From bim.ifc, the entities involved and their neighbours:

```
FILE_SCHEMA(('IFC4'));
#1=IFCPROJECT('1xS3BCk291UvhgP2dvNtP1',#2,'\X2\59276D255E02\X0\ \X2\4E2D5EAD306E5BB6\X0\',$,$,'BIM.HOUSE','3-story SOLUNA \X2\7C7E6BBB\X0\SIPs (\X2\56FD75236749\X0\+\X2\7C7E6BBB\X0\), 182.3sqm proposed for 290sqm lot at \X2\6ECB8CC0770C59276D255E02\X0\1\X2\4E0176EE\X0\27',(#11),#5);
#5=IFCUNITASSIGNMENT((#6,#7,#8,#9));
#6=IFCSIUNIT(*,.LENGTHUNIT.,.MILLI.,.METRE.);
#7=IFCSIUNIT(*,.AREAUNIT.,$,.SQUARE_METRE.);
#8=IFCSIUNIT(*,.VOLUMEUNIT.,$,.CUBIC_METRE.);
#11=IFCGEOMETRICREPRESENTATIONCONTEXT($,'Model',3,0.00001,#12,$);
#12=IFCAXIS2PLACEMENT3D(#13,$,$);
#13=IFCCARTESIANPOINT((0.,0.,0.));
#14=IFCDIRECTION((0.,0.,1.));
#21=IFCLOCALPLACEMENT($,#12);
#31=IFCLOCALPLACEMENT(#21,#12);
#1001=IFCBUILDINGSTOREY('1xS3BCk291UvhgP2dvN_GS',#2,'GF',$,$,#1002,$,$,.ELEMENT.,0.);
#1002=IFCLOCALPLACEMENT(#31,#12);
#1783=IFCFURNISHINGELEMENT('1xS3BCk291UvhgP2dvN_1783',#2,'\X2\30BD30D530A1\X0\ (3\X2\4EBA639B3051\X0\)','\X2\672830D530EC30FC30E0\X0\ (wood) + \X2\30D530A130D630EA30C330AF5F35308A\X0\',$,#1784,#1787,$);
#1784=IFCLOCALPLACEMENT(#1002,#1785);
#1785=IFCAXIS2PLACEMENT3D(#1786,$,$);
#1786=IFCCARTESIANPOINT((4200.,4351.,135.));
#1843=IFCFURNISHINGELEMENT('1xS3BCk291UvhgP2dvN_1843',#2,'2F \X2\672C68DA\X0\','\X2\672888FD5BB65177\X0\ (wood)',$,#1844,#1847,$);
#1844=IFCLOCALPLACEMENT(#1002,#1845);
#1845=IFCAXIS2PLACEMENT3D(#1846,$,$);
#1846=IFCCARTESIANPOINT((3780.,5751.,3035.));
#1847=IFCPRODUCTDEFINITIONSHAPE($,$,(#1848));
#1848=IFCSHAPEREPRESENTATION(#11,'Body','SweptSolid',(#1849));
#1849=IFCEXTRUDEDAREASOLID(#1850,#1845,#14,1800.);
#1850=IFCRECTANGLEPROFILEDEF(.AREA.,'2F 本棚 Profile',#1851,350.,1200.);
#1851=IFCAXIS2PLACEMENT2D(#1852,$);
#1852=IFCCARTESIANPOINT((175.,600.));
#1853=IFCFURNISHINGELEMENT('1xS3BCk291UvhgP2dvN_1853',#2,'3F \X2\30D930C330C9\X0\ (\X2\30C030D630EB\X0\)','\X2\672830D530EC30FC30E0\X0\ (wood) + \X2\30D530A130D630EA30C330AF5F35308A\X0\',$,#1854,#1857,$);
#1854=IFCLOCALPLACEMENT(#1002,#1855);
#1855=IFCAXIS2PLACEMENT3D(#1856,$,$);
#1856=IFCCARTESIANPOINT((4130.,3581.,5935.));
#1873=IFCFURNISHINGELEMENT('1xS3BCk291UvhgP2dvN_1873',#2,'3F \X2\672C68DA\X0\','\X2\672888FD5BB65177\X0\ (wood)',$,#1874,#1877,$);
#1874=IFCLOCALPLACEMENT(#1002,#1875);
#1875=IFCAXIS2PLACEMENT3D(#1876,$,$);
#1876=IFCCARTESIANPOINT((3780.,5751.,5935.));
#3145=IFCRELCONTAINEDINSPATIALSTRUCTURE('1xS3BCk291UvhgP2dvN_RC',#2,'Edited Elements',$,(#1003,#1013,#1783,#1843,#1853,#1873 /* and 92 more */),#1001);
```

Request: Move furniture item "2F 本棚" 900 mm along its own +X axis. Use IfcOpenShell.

```python
import ifcopenshell
import ifcopenshell.api.geometry
import ifcopenshell.util.placement
import ifcopenshell.util.unit

model = ifcopenshell.open("bim.ifc")
unit_scale = ifcopenshell.util.unit.calculate_unit_scale(model)

item = model.by_guid("1xS3BCk291UvhgP2dvN_1843")
matrix = ifcopenshell.util.placement.get_local_placement(item.ObjectPlacement)
matrix[:3, 3] += matrix[:3, 0] * 0.9 / unit_scale
ifcopenshell.api.geometry.edit_object_placement(model, product=item, matrix=matrix, is_si=False)

print(ifcopenshell.util.placement.get_local_placement(item.ObjectPlacement).round(3) + 0.0)

model.write("bim_edited.ifc")
```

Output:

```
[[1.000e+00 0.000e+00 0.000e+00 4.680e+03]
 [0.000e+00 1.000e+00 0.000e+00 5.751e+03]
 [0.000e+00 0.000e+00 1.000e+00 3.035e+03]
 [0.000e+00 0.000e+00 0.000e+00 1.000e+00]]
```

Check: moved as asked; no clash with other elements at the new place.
